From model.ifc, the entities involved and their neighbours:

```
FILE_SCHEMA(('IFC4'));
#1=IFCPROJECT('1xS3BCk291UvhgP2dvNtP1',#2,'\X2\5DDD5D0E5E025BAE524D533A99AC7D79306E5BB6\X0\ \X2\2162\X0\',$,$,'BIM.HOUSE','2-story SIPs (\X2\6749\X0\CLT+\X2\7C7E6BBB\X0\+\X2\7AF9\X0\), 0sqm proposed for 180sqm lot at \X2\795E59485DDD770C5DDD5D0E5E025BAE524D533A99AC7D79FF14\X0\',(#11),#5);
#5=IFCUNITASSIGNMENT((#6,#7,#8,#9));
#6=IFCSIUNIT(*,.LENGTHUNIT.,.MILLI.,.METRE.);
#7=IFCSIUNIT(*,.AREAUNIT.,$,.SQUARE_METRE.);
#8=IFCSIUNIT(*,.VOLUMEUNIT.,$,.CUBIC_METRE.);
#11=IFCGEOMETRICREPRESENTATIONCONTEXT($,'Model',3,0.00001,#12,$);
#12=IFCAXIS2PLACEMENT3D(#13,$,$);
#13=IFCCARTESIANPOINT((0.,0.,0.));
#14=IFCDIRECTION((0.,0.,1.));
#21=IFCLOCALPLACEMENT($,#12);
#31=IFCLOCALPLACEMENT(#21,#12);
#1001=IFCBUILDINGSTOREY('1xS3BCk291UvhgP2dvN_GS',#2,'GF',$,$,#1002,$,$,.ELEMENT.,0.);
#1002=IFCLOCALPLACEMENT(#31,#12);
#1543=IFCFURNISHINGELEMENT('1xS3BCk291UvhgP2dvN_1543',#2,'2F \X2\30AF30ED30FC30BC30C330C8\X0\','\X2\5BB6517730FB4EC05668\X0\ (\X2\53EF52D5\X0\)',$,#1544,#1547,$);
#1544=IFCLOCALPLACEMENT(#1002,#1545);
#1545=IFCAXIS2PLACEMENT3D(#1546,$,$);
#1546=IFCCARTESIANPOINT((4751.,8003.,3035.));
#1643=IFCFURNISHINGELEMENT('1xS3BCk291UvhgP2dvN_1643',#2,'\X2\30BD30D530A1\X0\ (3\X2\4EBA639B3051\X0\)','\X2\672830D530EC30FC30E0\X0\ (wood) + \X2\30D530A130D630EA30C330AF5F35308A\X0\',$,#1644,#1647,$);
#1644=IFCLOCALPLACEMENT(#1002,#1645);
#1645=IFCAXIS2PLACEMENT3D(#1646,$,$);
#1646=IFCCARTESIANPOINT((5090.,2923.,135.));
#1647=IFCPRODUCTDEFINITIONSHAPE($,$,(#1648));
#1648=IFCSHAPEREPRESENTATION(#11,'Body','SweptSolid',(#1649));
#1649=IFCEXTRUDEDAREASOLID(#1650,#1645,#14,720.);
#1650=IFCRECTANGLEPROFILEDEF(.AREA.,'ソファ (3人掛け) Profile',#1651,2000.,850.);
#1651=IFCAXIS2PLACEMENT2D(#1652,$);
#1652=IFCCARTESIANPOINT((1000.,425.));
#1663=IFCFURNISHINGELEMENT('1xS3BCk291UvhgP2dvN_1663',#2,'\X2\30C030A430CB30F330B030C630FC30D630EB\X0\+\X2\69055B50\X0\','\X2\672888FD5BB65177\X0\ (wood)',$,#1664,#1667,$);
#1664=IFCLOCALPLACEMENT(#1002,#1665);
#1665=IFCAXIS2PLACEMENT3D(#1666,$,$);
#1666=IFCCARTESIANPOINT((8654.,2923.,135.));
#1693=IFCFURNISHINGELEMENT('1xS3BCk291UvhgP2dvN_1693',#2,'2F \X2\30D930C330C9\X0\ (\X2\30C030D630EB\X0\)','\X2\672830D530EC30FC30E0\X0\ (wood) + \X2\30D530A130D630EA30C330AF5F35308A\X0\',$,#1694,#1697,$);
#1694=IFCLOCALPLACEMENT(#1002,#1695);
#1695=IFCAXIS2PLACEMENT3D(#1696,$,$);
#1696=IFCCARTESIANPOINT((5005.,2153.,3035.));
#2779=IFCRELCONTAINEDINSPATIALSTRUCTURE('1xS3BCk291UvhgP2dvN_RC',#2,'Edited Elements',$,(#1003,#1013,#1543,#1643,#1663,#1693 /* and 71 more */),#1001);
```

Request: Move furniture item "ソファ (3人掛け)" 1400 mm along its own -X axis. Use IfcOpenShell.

```python
import ifcopenshell
import ifcopenshell.api.geometry
import ifcopenshell.util.placement

model = ifcopenshell.open("model.ifc")

item = model.by_guid("1xS3BCk291UvhgP2dvN_1643")
matrix = ifcopenshell.util.placement.get_local_placement(item.ObjectPlacement)
matrix[:3, 3] -= matrix[:3, 0] * 1400.0
ifcopenshell.api.geometry.edit_object_placement(model, product=item, matrix=matrix, is_si=False)

print(ifcopenshell.util.placement.get_local_placement(item.ObjectPlacement).round(3) + 0.0)

model.write("model_edited.ifc")
```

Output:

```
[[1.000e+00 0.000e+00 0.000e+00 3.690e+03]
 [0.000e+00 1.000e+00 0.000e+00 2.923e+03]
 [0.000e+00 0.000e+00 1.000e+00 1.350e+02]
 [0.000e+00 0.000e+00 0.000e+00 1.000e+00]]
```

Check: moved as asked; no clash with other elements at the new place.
